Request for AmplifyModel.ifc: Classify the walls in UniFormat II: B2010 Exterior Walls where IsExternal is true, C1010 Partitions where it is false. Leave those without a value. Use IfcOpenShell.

First a look at what the model holds.

```python
import ifcopenshell
import ifcopenshell.util.element

model = ifcopenshell.open("AmplifyModel.ifc")
print(model.schema)
print("classifications:", [c.Name for c in model.by_type("IfcClassification")])
values = [ifcopenshell.util.element.get_pset(e, "Pset_WallCommon", "IsExternal") for e in model.by_type("IfcWall")]
for value in (True, False, None):
    print("IsExternal", value, values.count(value))
```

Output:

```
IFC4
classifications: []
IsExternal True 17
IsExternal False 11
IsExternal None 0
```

```python
import ifcopenshell
import ifcopenshell.api.classification
import ifcopenshell.util.element

model = ifcopenshell.open("AmplifyModel.ifc")

system = ifcopenshell.api.classification.add_classification(model, classification="UniFormat II")

walls = model.by_type("IfcWall")
external = {e: ifcopenshell.util.element.get_pset(e, "Pset_WallCommon", "IsExternal") for e in walls}
for flag, code, name in ((True, "B2010", "Exterior Walls"), (False, "C1010", "Partitions")):
    products = [e for e in walls if external[e] is flag]
    ifcopenshell.api.classification.add_reference(
        model, products=products, classification=system, identification=code, name=name
    )
    print(code, len(products))

model.write("AmplifyModel_v2.ifc")
```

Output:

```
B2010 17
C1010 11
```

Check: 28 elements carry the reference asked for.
